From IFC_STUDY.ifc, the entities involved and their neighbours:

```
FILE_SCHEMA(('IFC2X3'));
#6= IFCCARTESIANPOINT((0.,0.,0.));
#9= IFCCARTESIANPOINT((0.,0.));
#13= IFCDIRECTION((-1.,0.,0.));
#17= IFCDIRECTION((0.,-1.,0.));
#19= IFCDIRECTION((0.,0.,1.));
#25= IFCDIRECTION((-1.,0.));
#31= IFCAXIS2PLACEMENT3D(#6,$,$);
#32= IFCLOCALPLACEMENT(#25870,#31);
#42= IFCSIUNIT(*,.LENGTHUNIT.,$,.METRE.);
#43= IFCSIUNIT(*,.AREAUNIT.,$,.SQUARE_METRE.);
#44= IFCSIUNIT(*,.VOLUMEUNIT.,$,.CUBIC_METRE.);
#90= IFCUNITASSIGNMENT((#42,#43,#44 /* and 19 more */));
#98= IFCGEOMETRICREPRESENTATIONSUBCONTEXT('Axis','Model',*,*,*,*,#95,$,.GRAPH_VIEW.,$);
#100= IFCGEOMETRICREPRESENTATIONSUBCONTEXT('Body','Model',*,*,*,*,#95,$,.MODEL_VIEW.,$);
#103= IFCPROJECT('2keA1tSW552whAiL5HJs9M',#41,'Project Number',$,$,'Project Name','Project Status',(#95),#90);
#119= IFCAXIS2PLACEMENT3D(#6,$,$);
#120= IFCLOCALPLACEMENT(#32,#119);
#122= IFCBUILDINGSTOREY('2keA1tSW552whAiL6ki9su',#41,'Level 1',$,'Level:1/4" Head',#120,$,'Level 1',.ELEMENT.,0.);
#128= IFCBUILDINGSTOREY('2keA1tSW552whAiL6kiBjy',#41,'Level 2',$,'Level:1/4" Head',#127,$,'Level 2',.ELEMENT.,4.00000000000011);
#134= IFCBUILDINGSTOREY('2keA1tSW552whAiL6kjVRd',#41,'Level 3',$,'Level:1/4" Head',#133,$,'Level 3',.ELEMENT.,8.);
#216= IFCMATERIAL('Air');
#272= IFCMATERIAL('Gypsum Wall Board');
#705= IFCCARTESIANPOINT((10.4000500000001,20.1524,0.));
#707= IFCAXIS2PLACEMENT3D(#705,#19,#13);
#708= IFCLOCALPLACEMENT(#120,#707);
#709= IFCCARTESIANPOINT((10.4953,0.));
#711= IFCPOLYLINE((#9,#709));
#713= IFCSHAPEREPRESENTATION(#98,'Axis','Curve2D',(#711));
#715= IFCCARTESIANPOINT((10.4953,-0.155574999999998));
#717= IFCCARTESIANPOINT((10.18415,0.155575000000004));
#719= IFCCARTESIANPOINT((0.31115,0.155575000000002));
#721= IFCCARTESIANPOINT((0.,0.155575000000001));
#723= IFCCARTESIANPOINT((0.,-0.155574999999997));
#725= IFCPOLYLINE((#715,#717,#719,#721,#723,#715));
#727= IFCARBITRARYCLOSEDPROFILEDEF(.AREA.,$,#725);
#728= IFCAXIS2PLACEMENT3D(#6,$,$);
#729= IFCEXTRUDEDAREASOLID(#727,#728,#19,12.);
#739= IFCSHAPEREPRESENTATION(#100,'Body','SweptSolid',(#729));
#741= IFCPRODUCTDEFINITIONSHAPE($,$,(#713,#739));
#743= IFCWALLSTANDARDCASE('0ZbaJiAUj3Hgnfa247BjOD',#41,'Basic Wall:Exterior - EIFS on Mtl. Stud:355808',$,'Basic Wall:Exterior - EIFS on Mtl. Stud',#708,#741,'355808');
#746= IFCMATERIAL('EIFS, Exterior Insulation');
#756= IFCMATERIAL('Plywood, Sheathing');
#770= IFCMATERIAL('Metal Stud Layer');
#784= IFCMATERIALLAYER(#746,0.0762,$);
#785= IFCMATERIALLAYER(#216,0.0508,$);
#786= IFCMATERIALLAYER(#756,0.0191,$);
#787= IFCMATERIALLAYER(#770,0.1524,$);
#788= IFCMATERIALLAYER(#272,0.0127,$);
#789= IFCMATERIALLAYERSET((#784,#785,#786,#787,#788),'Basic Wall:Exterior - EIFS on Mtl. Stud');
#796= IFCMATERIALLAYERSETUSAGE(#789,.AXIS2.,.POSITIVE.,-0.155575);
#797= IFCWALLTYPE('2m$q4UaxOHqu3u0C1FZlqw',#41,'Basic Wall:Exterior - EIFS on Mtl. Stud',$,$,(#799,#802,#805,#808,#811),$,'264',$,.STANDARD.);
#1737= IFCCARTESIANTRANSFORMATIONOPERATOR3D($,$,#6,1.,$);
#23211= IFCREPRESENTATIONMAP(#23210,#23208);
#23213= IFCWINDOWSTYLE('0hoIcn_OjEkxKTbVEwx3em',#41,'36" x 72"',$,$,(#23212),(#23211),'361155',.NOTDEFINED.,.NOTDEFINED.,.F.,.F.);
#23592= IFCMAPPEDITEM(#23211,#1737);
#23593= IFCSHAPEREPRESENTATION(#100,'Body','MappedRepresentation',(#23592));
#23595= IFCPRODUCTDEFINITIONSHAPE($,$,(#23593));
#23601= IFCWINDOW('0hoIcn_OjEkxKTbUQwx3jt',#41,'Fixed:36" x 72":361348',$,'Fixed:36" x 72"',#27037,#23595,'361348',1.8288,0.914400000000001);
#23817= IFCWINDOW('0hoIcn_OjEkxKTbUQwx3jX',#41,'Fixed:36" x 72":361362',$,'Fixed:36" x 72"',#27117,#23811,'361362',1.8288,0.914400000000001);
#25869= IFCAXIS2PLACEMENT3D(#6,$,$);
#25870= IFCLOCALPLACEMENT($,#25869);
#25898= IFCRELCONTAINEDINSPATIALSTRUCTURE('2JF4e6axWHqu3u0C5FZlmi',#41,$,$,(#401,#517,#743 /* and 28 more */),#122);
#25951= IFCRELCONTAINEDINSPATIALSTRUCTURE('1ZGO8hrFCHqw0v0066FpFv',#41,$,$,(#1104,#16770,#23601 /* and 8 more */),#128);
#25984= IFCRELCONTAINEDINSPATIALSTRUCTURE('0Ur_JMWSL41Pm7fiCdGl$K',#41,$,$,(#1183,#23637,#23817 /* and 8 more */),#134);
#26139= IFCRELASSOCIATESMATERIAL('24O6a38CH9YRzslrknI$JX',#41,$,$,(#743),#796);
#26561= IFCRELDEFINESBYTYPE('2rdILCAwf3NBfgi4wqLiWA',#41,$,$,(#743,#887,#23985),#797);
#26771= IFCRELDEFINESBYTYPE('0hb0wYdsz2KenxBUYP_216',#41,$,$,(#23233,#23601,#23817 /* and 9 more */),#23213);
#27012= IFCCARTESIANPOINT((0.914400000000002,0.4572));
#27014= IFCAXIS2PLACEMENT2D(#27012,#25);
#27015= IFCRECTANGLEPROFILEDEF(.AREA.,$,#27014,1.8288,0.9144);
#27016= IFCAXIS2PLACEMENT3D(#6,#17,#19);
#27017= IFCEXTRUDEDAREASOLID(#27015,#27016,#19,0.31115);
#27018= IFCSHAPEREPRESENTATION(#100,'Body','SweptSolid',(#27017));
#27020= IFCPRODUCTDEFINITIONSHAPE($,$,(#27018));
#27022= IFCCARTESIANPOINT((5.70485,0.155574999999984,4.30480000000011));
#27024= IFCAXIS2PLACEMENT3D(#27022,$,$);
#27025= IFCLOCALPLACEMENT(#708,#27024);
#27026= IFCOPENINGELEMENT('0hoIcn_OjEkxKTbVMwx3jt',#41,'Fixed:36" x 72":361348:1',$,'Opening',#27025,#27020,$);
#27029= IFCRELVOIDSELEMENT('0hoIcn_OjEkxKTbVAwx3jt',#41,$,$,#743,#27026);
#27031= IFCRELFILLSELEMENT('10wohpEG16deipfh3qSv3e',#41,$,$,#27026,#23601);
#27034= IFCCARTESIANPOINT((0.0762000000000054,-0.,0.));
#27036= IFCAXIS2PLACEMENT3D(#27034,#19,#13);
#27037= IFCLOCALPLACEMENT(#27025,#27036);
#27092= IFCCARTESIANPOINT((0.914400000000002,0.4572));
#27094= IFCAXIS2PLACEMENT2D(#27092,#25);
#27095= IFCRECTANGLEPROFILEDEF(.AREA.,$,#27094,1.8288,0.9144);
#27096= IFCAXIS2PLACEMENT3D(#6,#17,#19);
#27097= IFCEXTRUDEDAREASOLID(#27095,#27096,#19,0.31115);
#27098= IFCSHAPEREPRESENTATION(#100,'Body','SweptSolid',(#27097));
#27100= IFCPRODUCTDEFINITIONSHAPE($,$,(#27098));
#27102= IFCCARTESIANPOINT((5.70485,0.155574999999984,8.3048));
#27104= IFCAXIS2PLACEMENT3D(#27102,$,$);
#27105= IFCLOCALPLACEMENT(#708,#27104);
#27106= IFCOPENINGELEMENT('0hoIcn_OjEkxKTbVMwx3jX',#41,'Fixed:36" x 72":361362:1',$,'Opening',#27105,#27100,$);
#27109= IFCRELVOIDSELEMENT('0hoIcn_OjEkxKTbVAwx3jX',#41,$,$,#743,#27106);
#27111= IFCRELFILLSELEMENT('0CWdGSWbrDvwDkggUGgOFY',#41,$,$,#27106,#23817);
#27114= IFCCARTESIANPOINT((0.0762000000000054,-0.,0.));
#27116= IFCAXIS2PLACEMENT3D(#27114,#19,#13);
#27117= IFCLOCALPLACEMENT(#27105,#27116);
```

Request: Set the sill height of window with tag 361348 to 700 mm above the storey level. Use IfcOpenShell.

```python
import numpy as np
import ifcopenshell
import ifcopenshell.api.geometry
import ifcopenshell.geom
import ifcopenshell.util.element
import ifcopenshell.util.placement
import ifcopenshell.util.shape
import ifcopenshell.util.unit

model = ifcopenshell.open("IFC_STUDY.ifc")
unit_scale = ifcopenshell.util.unit.calculate_unit_scale(model)

window = model.by_id(23601)
opening = window.FillsVoids[0].RelatingOpeningElement
storey = ifcopenshell.util.element.get_container(window, ifc_class="IfcBuildingStorey")
level = ifcopenshell.util.placement.get_local_placement(storey.ObjectPlacement)[2, 3]

# The opening's origin need not be at the sill, so measure its lowest point.
shape = ifcopenshell.geom.create_shape(ifcopenshell.geom.settings(), opening)
bottom = ifcopenshell.util.shape.get_shape_bottom_elevation(shape, shape.geometry) / unit_scale
dz = level + 0.7 / unit_scale - bottom

shift = np.array([0.0, 0.0, dz])
# The window is placed relative to its opening, so it follows when the opening moves.
matrix = ifcopenshell.util.placement.get_local_placement(opening.ObjectPlacement)
matrix[:3, 3] += shift
ifcopenshell.api.geometry.edit_object_placement(
    model, product=opening, matrix=matrix, is_si=False, should_transform_children=True
)

print(f"moved by {dz * unit_scale:+.3f} m")

model.write("IFC_STUDY_rev.ifc")
```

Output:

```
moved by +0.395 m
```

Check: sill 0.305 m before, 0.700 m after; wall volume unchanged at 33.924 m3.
